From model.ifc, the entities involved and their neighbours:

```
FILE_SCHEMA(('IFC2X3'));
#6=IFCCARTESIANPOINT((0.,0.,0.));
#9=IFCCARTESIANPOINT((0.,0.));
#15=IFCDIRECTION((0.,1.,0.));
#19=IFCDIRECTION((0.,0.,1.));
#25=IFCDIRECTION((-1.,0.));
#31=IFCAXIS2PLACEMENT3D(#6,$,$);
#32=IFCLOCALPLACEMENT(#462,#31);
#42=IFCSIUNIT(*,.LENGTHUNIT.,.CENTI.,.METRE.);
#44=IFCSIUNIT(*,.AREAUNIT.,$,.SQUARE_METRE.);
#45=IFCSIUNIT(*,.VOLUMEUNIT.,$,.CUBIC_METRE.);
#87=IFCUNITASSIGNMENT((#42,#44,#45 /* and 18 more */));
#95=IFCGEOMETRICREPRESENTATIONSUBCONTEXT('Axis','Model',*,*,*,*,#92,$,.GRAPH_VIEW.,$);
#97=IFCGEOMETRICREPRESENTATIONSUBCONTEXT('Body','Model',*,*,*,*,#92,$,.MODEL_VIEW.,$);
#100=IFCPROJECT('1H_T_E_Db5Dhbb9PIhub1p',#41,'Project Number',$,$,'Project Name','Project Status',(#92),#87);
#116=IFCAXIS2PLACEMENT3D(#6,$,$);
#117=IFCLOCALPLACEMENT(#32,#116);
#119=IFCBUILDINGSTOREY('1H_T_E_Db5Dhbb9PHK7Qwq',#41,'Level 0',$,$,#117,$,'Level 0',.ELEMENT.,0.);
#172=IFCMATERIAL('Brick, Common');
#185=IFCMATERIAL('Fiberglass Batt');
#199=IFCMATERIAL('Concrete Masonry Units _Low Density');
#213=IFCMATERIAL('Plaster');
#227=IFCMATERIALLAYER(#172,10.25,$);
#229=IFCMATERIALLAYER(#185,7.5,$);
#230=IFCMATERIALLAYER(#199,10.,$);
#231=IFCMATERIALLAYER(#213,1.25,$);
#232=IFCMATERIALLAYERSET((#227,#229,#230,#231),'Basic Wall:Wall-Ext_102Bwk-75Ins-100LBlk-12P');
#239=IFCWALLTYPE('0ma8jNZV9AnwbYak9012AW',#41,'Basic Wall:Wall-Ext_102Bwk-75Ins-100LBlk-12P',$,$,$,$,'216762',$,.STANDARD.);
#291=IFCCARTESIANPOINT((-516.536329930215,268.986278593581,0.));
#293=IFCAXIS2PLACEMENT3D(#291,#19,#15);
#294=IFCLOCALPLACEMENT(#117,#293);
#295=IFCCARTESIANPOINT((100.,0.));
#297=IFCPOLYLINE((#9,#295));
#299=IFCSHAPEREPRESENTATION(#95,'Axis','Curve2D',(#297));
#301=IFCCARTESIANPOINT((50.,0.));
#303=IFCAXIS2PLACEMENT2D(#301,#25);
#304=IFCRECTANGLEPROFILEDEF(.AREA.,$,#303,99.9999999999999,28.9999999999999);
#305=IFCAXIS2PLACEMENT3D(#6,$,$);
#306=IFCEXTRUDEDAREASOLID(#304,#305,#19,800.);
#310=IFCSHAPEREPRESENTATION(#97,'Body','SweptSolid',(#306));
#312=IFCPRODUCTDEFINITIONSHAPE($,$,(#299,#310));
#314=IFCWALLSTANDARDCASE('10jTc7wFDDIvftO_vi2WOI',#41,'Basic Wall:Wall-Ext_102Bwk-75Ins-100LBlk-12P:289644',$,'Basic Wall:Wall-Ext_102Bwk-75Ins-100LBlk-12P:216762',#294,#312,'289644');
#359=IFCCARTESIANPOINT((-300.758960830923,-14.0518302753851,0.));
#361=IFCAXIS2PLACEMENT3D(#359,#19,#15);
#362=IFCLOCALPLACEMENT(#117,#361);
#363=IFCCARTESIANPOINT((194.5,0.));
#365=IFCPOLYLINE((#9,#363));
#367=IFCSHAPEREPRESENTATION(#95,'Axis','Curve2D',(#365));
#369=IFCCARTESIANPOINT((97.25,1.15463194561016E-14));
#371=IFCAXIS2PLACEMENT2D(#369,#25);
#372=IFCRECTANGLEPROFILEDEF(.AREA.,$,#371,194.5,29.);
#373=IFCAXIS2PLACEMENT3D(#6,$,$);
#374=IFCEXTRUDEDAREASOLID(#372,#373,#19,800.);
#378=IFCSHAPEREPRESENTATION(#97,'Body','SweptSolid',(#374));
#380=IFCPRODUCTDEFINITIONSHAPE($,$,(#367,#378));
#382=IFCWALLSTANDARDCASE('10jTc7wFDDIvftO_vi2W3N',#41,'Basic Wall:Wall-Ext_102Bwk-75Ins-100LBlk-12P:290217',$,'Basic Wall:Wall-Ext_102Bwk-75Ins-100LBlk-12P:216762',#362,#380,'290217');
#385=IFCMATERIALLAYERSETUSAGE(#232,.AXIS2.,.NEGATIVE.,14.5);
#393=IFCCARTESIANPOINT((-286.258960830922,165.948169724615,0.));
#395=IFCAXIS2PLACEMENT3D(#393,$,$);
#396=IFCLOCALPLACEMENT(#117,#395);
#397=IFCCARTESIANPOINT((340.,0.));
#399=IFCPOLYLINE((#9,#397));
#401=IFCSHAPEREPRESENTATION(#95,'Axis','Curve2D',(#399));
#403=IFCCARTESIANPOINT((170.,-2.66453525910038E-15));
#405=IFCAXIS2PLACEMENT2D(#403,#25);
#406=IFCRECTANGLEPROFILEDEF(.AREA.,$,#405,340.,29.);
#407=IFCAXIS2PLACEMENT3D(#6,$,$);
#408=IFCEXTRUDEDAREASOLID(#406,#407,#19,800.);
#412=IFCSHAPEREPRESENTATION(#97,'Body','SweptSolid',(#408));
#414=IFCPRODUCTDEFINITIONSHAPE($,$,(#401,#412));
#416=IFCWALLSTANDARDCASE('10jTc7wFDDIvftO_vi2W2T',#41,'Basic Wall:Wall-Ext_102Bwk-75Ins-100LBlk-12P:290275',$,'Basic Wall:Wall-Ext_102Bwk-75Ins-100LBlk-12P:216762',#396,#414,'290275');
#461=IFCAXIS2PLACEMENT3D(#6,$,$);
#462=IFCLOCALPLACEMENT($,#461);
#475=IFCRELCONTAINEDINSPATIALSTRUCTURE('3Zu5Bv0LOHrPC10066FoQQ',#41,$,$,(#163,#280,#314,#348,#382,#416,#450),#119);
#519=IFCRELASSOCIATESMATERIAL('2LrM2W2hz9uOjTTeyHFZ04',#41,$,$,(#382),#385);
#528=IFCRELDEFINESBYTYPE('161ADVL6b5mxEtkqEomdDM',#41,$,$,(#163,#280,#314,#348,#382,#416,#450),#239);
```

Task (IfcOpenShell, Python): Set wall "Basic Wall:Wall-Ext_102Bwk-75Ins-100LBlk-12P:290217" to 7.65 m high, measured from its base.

```python
import ifcopenshell
import ifcopenshell.geom
import ifcopenshell.util.representation
import ifcopenshell.util.shape
import ifcopenshell.util.unit

model = ifcopenshell.open("model.ifc")
unit_scale = ifcopenshell.util.unit.calculate_unit_scale(model)
settings = ifcopenshell.geom.settings()


def volume(element):
    """Net volume in cubic metres, openings subtracted."""
    shape = ifcopenshell.geom.create_shape(settings, element)
    return ifcopenshell.util.shape.get_volume(shape.geometry)


wall = model.by_guid("10jTc7wFDDIvftO_vi2W3N")
before = volume(wall)

body = ifcopenshell.util.representation.get_representation(wall, "Model", "Body")
solid = body.Items[0]
old_height = solid.Depth
solid.Depth = 7.65 / unit_scale
after = volume(wall)

print(f"height {old_height:g} -> {solid.Depth:g}, volume {before:.3f} -> {after:.3f} m3")

model.write("model_updated.ifc")
```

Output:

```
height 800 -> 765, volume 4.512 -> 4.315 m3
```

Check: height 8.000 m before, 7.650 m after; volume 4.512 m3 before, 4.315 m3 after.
